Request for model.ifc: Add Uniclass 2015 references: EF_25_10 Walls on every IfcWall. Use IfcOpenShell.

First a look at what the model holds.

```python
import ifcopenshell

model = ifcopenshell.open("model.ifc")
print(model.schema)
print("classifications:", [c.Name for c in model.by_type("IfcClassification")])
for ifc_class in ("IfcDoor", "IfcRoof", "IfcStair", "IfcWall", "IfcWindow"):
    print(ifc_class, len(model.by_type(ifc_class)))
```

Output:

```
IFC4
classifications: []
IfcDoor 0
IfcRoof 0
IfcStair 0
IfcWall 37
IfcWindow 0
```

```python
import ifcopenshell
import ifcopenshell.api.classification

model = ifcopenshell.open("model.ifc")

system = ifcopenshell.api.classification.add_classification(model, classification="Uniclass 2015")

codes = {
    "IfcWall": ("EF_25_10", "Walls"),
}
for ifc_class, (code, name) in codes.items():
    products = model.by_type(ifc_class)
    ifcopenshell.api.classification.add_reference(
        model, products=products, classification=system, identification=code, name=name
    )
    print(code, len(products))

model.write("model_edited.ifc")
```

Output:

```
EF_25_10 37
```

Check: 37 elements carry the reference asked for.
